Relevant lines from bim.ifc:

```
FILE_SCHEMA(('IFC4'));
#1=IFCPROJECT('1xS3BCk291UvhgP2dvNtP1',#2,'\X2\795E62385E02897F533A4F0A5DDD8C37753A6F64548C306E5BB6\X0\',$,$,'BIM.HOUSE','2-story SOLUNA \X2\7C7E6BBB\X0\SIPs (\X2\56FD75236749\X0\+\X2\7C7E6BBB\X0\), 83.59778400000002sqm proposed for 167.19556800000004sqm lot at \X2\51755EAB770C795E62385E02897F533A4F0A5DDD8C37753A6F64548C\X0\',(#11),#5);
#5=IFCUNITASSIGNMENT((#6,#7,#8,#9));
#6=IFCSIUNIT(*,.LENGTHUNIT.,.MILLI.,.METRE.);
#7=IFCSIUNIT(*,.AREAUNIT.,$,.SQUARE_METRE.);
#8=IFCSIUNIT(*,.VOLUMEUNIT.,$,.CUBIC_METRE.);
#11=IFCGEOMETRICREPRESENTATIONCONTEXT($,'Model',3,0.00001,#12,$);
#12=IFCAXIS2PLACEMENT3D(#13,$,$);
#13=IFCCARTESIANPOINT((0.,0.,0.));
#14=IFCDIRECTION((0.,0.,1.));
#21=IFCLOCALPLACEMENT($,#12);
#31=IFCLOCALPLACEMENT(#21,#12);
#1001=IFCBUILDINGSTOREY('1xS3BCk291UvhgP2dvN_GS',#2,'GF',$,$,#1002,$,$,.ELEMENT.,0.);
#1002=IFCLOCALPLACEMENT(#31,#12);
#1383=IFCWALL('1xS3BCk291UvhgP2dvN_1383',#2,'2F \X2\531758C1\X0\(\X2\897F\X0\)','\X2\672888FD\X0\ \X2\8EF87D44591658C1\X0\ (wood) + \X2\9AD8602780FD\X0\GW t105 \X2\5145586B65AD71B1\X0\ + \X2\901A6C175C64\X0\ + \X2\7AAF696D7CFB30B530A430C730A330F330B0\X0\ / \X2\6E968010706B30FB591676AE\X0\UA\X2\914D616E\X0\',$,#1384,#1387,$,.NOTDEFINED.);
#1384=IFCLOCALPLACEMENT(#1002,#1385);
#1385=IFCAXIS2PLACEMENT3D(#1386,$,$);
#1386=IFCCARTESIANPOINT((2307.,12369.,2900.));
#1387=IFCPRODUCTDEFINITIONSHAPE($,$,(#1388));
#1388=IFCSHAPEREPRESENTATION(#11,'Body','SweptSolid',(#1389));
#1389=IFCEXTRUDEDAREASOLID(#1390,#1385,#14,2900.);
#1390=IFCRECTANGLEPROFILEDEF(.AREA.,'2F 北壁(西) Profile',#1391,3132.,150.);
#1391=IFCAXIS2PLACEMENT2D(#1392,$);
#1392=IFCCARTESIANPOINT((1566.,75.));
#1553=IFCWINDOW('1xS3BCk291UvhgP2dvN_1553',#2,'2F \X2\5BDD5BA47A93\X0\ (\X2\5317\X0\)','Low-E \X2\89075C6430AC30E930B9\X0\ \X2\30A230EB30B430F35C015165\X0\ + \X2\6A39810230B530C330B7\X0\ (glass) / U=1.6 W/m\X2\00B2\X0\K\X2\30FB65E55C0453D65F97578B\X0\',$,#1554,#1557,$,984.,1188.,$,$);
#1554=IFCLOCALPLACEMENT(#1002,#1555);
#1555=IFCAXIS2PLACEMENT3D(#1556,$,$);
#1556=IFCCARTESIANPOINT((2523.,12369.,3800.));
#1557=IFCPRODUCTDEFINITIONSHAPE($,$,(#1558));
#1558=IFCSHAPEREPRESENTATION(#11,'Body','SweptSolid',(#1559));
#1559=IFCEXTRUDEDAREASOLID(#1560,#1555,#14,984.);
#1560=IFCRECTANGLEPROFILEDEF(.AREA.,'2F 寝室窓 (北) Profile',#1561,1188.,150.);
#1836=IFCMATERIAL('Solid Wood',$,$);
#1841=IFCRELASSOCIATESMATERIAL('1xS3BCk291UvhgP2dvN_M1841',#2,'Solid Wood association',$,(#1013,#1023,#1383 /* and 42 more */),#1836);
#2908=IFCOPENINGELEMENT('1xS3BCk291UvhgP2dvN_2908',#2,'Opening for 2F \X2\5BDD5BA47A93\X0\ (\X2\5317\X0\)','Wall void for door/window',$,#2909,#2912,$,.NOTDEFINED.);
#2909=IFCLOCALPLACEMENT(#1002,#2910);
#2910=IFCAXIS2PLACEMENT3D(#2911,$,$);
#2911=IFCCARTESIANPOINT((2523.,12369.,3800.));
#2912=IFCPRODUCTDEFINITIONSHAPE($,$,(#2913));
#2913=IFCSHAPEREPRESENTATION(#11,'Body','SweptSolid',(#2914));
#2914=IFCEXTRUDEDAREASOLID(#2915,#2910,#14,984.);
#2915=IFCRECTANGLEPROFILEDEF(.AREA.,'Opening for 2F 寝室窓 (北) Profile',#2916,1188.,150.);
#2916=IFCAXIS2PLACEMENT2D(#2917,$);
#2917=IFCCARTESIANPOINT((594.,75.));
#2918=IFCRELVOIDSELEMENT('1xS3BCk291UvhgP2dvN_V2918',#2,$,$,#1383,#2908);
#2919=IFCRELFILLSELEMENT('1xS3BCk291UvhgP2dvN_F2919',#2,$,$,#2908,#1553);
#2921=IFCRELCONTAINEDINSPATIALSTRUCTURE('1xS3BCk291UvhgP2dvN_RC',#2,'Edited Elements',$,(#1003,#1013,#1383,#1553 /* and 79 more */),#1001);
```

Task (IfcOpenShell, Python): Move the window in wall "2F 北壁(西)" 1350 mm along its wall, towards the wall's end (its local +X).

```python
import ifcopenshell
import ifcopenshell.api.geometry
import ifcopenshell.util.placement

model = ifcopenshell.open("bim.ifc")

window = model.by_guid("1xS3BCk291UvhgP2dvN_1553")
opening = window.FillsVoids[0].RelatingOpeningElement
wall = opening.VoidsElements[0].RelatingBuildingElement

wall_matrix = ifcopenshell.util.placement.get_local_placement(wall.ObjectPlacement)
shift = wall_matrix[:3, 0] * 1350.0
before = ifcopenshell.util.placement.get_local_placement(window.ObjectPlacement)[:3, 3].copy()

# The window is not placed relative to its opening, so move both.
for product in (opening, window):
    matrix = ifcopenshell.util.placement.get_local_placement(product.ObjectPlacement)
    matrix[:3, 3] += shift
    ifcopenshell.api.geometry.edit_object_placement(model, product=product, matrix=matrix, is_si=False)

after = ifcopenshell.util.placement.get_local_placement(window.ObjectPlacement)[:3, 3]
print("window moved by", (after - before).round(3) + 0.0)

model.write("bim_v2.ifc")
```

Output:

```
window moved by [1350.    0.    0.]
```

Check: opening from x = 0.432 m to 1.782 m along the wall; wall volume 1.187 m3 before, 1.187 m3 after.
